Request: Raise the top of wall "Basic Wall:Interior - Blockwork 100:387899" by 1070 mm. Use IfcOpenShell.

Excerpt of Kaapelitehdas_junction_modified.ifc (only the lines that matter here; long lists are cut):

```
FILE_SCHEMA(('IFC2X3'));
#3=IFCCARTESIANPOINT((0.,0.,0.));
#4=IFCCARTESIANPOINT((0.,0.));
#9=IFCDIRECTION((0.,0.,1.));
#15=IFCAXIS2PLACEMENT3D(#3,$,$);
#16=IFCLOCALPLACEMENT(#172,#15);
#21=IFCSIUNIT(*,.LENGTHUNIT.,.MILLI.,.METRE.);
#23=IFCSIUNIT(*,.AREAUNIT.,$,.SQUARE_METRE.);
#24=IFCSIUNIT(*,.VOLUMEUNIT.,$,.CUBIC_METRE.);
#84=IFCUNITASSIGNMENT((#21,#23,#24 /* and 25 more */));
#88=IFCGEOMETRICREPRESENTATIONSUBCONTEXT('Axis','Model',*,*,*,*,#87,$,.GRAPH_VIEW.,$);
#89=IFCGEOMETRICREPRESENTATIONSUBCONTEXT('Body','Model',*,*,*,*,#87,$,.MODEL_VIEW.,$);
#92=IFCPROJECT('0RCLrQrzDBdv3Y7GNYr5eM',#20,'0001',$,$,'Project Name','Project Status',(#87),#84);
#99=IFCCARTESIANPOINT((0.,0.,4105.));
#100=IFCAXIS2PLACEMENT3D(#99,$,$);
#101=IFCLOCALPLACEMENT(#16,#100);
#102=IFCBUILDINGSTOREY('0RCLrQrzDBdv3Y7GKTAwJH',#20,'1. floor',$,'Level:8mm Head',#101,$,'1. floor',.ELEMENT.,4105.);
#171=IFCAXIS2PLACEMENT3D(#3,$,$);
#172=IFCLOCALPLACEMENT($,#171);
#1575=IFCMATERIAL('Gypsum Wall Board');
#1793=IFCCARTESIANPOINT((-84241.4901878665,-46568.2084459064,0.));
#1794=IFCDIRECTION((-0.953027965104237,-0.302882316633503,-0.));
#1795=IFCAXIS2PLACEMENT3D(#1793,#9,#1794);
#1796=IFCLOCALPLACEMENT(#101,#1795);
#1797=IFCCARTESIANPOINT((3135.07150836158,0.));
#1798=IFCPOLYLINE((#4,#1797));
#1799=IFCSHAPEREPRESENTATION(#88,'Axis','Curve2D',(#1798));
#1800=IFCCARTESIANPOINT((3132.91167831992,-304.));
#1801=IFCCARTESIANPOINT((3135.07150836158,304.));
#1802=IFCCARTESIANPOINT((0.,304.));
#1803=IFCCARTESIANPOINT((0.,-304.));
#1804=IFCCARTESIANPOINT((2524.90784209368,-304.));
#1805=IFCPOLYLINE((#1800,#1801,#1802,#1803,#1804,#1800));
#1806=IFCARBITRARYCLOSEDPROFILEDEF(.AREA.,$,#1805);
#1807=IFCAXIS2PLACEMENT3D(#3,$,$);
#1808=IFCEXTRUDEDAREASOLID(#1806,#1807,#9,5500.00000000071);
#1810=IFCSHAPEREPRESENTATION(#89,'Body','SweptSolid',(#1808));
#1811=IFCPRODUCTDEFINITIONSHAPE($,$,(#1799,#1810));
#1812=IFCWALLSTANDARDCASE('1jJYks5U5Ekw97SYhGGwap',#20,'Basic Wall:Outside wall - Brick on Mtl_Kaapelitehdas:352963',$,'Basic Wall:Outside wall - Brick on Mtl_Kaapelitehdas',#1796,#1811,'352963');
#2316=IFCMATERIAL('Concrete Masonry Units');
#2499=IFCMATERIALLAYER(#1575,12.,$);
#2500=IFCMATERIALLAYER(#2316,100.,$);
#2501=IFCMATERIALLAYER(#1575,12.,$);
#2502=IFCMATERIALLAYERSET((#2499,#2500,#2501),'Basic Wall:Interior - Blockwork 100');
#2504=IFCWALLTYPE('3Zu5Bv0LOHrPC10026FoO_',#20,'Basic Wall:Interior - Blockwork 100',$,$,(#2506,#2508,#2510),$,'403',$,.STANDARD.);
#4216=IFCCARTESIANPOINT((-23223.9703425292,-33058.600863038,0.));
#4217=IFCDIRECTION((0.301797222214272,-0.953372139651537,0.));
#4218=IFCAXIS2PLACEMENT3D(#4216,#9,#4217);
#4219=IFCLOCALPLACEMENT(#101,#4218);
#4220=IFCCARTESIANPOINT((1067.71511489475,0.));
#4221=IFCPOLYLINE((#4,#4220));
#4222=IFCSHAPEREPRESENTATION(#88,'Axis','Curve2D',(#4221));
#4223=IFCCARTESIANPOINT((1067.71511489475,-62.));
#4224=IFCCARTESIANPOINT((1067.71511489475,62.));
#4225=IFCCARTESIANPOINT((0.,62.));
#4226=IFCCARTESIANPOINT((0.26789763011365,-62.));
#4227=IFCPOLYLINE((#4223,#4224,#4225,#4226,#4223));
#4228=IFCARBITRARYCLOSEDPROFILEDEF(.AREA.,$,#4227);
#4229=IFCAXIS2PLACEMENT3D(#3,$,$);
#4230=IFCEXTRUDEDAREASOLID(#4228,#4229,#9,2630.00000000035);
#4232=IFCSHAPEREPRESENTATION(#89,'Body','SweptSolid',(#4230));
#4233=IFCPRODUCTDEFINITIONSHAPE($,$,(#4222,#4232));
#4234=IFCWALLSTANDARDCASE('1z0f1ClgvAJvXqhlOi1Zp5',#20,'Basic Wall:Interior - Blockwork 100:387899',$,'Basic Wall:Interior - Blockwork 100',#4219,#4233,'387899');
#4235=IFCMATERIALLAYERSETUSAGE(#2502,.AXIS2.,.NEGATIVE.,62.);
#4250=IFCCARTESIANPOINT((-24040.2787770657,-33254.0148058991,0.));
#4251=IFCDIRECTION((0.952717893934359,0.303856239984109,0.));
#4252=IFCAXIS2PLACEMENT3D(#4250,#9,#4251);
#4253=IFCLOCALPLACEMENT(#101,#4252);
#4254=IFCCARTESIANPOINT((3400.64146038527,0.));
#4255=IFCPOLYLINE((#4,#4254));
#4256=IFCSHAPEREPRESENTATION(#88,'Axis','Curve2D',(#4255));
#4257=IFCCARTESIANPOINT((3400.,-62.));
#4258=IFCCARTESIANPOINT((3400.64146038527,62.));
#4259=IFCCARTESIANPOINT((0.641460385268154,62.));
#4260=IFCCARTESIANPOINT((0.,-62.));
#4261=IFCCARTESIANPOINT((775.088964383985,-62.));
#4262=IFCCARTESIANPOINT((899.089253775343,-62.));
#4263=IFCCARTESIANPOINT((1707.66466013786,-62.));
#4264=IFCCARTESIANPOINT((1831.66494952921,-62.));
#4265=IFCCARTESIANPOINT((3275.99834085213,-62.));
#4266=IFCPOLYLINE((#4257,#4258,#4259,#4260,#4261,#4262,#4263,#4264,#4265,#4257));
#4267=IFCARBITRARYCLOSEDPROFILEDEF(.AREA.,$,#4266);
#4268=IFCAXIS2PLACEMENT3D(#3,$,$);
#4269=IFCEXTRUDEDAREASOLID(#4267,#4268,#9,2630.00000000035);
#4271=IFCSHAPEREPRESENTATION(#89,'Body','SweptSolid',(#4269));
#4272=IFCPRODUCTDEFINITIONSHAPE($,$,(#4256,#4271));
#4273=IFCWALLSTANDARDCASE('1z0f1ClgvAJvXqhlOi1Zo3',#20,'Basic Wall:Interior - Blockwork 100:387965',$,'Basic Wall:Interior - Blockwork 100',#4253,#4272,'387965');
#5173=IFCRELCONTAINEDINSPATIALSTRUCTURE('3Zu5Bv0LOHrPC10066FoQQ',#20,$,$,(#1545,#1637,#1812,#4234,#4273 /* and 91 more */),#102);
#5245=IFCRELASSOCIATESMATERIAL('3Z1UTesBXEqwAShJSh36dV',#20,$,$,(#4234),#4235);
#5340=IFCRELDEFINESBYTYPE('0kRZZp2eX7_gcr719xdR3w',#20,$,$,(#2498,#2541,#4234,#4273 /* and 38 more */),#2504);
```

```python
import ifcopenshell
import ifcopenshell.geom
import ifcopenshell.util.representation
import ifcopenshell.util.shape
import ifcopenshell.util.unit

model = ifcopenshell.open("Kaapelitehdas_junction_modified.ifc")
unit_scale = ifcopenshell.util.unit.calculate_unit_scale(model)
settings = ifcopenshell.geom.settings()


def volume(element):
    """Net volume in cubic metres, openings subtracted."""
    shape = ifcopenshell.geom.create_shape(settings, element)
    return ifcopenshell.util.shape.get_volume(shape.geometry)


wall = model.by_guid("1z0f1ClgvAJvXqhlOi1Zp5")
before = volume(wall)

body = ifcopenshell.util.representation.get_representation(wall, "Model", "Body")
solid = body.Items[0]
old_height = solid.Depth
solid.Depth += 1.07 / unit_scale
after = volume(wall)

print(f"height {old_height:g} -> {solid.Depth:g}, volume {before:.3f} -> {after:.3f} m3")

model.write("Kaapelitehdas_junction_modified_updated.ifc")
```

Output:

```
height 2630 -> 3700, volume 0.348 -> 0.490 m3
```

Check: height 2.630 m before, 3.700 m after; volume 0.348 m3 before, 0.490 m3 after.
